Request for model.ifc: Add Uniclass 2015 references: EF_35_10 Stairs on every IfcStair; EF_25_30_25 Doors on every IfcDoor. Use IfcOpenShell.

First a look at what the model holds.

```python
import ifcopenshell

model = ifcopenshell.open("model.ifc")
print(model.schema)
print("classifications:", [c.Name for c in model.by_type("IfcClassification")])
for ifc_class in ("IfcDoor", "IfcRoof", "IfcStair", "IfcWall", "IfcWindow"):
    print(ifc_class, len(model.by_type(ifc_class)))
```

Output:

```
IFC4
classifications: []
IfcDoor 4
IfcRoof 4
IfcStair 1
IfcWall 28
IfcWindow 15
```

```python
import ifcopenshell
import ifcopenshell.api.classification

model = ifcopenshell.open("model.ifc")

system = ifcopenshell.api.classification.add_classification(model, classification="Uniclass 2015")

codes = {
    "IfcStair": ("EF_35_10", "Stairs"),
    "IfcDoor": ("EF_25_30_25", "Doors"),
}
for ifc_class, (code, name) in codes.items():
    products = model.by_type(ifc_class)
    ifcopenshell.api.classification.add_reference(
        model, products=products, classification=system, identification=code, name=name
    )
    print(code, len(products))

model.write("model_edited.ifc")
```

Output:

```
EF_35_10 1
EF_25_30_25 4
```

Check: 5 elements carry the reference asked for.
